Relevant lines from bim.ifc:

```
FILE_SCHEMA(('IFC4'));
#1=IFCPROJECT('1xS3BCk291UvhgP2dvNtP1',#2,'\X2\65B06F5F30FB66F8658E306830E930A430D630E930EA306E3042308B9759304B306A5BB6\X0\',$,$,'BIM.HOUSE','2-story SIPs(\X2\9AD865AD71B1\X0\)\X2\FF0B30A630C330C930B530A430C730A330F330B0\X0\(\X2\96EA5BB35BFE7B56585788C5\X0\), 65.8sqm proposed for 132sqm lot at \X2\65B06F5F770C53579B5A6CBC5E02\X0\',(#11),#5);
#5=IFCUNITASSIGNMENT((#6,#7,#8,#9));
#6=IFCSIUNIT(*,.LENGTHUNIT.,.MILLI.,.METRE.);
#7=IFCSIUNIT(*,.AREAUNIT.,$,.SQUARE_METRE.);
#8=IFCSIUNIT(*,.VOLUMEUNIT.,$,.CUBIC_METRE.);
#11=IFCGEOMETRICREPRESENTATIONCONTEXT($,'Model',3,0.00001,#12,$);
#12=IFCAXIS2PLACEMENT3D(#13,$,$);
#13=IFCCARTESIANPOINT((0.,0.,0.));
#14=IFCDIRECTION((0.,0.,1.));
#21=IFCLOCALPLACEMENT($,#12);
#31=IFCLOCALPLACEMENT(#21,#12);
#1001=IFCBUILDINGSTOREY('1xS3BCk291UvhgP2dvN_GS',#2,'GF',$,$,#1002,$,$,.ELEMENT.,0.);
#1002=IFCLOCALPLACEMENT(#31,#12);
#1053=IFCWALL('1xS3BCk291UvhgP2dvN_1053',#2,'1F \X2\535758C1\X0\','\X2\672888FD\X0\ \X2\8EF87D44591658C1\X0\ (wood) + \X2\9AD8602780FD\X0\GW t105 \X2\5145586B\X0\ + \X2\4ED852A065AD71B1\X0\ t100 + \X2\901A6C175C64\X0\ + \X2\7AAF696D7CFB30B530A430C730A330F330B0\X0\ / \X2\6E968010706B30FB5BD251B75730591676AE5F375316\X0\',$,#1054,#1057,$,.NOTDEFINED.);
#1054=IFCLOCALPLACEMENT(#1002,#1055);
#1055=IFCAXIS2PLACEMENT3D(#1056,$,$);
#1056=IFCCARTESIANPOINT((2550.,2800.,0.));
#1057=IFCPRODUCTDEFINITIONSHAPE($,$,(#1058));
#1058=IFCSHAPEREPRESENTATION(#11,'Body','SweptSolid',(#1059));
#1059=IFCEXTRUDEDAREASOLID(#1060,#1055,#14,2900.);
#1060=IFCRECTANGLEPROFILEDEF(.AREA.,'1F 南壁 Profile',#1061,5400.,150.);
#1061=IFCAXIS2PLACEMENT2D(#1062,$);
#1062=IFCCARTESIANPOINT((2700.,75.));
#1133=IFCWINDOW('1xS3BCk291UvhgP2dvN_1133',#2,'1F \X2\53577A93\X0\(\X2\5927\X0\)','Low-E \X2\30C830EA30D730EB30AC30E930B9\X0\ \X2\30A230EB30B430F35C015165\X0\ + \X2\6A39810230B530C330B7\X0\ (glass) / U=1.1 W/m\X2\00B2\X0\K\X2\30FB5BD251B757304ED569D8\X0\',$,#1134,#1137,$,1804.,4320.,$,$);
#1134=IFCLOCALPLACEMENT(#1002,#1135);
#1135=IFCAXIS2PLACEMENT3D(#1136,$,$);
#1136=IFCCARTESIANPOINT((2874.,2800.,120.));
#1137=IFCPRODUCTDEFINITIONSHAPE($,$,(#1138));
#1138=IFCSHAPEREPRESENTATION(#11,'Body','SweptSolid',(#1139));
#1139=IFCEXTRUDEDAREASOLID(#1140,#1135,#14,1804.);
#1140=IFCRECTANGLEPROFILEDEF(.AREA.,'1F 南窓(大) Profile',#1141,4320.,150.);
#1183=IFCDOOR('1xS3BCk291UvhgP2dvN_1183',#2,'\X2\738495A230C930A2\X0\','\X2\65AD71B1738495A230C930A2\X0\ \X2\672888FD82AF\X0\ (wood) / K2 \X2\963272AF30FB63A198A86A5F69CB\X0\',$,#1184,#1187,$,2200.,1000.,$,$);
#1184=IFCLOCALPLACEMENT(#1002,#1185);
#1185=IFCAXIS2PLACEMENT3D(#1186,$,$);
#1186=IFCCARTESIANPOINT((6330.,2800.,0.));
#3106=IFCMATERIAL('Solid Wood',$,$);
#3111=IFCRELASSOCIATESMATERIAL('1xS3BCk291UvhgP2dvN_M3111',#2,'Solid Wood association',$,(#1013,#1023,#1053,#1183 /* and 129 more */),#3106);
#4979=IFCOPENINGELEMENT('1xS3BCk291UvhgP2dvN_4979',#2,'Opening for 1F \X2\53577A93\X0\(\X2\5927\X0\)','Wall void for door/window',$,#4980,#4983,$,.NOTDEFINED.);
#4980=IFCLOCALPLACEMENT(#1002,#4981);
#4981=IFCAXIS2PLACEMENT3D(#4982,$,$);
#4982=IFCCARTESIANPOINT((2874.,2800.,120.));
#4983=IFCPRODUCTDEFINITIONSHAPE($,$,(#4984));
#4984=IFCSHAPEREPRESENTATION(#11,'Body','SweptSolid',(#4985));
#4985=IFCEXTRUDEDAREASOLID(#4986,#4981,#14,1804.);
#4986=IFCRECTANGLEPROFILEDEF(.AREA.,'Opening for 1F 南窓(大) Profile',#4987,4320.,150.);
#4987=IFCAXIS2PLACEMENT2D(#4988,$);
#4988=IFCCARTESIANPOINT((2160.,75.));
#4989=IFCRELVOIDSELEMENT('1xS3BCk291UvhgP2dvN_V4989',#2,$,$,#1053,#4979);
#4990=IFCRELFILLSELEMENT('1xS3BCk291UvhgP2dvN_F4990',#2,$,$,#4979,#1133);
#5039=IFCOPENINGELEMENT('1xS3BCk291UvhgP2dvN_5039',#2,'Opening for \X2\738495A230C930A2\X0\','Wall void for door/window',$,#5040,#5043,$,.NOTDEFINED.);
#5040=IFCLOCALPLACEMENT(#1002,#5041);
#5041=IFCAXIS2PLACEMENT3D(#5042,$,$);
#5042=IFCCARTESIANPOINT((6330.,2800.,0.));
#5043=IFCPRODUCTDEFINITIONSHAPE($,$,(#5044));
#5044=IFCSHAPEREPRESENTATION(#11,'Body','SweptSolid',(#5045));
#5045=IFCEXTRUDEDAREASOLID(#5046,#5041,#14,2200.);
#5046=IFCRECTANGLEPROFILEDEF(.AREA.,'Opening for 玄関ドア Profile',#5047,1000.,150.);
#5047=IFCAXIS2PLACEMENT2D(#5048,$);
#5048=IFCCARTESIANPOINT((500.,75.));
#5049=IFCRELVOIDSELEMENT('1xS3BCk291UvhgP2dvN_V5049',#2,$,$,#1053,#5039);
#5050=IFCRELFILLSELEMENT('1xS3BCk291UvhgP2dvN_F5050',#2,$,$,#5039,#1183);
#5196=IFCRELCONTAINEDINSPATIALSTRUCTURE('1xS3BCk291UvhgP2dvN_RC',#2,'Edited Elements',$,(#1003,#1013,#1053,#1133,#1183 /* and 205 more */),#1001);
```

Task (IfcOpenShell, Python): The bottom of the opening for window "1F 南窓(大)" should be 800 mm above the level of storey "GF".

```python
import numpy as np
import ifcopenshell
import ifcopenshell.api.geometry
import ifcopenshell.geom
import ifcopenshell.util.element
import ifcopenshell.util.placement
import ifcopenshell.util.shape
import ifcopenshell.util.unit

model = ifcopenshell.open("bim.ifc")
unit_scale = ifcopenshell.util.unit.calculate_unit_scale(model)

window = model.by_id(1133)
opening = window.FillsVoids[0].RelatingOpeningElement
storey = ifcopenshell.util.element.get_container(window, ifc_class="IfcBuildingStorey")
level = ifcopenshell.util.placement.get_local_placement(storey.ObjectPlacement)[2, 3]

# The opening's origin need not be at the sill, so measure its lowest point.
shape = ifcopenshell.geom.create_shape(ifcopenshell.geom.settings(), opening)
bottom = ifcopenshell.util.shape.get_shape_bottom_elevation(shape, shape.geometry) / unit_scale
dz = level + 800.0 - bottom

shift = np.array([0.0, 0.0, dz])
# The window is not placed relative to its opening, so move both.
for product in (opening, window):
    matrix = ifcopenshell.util.placement.get_local_placement(product.ObjectPlacement)
    matrix[:3, 3] += shift
    ifcopenshell.api.geometry.edit_object_placement(model, product=product, matrix=matrix, is_si=False)

print(f"moved by {dz * unit_scale:+.3f} m")

model.write("bim-out.ifc")
```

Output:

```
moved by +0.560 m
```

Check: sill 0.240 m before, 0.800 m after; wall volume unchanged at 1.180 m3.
